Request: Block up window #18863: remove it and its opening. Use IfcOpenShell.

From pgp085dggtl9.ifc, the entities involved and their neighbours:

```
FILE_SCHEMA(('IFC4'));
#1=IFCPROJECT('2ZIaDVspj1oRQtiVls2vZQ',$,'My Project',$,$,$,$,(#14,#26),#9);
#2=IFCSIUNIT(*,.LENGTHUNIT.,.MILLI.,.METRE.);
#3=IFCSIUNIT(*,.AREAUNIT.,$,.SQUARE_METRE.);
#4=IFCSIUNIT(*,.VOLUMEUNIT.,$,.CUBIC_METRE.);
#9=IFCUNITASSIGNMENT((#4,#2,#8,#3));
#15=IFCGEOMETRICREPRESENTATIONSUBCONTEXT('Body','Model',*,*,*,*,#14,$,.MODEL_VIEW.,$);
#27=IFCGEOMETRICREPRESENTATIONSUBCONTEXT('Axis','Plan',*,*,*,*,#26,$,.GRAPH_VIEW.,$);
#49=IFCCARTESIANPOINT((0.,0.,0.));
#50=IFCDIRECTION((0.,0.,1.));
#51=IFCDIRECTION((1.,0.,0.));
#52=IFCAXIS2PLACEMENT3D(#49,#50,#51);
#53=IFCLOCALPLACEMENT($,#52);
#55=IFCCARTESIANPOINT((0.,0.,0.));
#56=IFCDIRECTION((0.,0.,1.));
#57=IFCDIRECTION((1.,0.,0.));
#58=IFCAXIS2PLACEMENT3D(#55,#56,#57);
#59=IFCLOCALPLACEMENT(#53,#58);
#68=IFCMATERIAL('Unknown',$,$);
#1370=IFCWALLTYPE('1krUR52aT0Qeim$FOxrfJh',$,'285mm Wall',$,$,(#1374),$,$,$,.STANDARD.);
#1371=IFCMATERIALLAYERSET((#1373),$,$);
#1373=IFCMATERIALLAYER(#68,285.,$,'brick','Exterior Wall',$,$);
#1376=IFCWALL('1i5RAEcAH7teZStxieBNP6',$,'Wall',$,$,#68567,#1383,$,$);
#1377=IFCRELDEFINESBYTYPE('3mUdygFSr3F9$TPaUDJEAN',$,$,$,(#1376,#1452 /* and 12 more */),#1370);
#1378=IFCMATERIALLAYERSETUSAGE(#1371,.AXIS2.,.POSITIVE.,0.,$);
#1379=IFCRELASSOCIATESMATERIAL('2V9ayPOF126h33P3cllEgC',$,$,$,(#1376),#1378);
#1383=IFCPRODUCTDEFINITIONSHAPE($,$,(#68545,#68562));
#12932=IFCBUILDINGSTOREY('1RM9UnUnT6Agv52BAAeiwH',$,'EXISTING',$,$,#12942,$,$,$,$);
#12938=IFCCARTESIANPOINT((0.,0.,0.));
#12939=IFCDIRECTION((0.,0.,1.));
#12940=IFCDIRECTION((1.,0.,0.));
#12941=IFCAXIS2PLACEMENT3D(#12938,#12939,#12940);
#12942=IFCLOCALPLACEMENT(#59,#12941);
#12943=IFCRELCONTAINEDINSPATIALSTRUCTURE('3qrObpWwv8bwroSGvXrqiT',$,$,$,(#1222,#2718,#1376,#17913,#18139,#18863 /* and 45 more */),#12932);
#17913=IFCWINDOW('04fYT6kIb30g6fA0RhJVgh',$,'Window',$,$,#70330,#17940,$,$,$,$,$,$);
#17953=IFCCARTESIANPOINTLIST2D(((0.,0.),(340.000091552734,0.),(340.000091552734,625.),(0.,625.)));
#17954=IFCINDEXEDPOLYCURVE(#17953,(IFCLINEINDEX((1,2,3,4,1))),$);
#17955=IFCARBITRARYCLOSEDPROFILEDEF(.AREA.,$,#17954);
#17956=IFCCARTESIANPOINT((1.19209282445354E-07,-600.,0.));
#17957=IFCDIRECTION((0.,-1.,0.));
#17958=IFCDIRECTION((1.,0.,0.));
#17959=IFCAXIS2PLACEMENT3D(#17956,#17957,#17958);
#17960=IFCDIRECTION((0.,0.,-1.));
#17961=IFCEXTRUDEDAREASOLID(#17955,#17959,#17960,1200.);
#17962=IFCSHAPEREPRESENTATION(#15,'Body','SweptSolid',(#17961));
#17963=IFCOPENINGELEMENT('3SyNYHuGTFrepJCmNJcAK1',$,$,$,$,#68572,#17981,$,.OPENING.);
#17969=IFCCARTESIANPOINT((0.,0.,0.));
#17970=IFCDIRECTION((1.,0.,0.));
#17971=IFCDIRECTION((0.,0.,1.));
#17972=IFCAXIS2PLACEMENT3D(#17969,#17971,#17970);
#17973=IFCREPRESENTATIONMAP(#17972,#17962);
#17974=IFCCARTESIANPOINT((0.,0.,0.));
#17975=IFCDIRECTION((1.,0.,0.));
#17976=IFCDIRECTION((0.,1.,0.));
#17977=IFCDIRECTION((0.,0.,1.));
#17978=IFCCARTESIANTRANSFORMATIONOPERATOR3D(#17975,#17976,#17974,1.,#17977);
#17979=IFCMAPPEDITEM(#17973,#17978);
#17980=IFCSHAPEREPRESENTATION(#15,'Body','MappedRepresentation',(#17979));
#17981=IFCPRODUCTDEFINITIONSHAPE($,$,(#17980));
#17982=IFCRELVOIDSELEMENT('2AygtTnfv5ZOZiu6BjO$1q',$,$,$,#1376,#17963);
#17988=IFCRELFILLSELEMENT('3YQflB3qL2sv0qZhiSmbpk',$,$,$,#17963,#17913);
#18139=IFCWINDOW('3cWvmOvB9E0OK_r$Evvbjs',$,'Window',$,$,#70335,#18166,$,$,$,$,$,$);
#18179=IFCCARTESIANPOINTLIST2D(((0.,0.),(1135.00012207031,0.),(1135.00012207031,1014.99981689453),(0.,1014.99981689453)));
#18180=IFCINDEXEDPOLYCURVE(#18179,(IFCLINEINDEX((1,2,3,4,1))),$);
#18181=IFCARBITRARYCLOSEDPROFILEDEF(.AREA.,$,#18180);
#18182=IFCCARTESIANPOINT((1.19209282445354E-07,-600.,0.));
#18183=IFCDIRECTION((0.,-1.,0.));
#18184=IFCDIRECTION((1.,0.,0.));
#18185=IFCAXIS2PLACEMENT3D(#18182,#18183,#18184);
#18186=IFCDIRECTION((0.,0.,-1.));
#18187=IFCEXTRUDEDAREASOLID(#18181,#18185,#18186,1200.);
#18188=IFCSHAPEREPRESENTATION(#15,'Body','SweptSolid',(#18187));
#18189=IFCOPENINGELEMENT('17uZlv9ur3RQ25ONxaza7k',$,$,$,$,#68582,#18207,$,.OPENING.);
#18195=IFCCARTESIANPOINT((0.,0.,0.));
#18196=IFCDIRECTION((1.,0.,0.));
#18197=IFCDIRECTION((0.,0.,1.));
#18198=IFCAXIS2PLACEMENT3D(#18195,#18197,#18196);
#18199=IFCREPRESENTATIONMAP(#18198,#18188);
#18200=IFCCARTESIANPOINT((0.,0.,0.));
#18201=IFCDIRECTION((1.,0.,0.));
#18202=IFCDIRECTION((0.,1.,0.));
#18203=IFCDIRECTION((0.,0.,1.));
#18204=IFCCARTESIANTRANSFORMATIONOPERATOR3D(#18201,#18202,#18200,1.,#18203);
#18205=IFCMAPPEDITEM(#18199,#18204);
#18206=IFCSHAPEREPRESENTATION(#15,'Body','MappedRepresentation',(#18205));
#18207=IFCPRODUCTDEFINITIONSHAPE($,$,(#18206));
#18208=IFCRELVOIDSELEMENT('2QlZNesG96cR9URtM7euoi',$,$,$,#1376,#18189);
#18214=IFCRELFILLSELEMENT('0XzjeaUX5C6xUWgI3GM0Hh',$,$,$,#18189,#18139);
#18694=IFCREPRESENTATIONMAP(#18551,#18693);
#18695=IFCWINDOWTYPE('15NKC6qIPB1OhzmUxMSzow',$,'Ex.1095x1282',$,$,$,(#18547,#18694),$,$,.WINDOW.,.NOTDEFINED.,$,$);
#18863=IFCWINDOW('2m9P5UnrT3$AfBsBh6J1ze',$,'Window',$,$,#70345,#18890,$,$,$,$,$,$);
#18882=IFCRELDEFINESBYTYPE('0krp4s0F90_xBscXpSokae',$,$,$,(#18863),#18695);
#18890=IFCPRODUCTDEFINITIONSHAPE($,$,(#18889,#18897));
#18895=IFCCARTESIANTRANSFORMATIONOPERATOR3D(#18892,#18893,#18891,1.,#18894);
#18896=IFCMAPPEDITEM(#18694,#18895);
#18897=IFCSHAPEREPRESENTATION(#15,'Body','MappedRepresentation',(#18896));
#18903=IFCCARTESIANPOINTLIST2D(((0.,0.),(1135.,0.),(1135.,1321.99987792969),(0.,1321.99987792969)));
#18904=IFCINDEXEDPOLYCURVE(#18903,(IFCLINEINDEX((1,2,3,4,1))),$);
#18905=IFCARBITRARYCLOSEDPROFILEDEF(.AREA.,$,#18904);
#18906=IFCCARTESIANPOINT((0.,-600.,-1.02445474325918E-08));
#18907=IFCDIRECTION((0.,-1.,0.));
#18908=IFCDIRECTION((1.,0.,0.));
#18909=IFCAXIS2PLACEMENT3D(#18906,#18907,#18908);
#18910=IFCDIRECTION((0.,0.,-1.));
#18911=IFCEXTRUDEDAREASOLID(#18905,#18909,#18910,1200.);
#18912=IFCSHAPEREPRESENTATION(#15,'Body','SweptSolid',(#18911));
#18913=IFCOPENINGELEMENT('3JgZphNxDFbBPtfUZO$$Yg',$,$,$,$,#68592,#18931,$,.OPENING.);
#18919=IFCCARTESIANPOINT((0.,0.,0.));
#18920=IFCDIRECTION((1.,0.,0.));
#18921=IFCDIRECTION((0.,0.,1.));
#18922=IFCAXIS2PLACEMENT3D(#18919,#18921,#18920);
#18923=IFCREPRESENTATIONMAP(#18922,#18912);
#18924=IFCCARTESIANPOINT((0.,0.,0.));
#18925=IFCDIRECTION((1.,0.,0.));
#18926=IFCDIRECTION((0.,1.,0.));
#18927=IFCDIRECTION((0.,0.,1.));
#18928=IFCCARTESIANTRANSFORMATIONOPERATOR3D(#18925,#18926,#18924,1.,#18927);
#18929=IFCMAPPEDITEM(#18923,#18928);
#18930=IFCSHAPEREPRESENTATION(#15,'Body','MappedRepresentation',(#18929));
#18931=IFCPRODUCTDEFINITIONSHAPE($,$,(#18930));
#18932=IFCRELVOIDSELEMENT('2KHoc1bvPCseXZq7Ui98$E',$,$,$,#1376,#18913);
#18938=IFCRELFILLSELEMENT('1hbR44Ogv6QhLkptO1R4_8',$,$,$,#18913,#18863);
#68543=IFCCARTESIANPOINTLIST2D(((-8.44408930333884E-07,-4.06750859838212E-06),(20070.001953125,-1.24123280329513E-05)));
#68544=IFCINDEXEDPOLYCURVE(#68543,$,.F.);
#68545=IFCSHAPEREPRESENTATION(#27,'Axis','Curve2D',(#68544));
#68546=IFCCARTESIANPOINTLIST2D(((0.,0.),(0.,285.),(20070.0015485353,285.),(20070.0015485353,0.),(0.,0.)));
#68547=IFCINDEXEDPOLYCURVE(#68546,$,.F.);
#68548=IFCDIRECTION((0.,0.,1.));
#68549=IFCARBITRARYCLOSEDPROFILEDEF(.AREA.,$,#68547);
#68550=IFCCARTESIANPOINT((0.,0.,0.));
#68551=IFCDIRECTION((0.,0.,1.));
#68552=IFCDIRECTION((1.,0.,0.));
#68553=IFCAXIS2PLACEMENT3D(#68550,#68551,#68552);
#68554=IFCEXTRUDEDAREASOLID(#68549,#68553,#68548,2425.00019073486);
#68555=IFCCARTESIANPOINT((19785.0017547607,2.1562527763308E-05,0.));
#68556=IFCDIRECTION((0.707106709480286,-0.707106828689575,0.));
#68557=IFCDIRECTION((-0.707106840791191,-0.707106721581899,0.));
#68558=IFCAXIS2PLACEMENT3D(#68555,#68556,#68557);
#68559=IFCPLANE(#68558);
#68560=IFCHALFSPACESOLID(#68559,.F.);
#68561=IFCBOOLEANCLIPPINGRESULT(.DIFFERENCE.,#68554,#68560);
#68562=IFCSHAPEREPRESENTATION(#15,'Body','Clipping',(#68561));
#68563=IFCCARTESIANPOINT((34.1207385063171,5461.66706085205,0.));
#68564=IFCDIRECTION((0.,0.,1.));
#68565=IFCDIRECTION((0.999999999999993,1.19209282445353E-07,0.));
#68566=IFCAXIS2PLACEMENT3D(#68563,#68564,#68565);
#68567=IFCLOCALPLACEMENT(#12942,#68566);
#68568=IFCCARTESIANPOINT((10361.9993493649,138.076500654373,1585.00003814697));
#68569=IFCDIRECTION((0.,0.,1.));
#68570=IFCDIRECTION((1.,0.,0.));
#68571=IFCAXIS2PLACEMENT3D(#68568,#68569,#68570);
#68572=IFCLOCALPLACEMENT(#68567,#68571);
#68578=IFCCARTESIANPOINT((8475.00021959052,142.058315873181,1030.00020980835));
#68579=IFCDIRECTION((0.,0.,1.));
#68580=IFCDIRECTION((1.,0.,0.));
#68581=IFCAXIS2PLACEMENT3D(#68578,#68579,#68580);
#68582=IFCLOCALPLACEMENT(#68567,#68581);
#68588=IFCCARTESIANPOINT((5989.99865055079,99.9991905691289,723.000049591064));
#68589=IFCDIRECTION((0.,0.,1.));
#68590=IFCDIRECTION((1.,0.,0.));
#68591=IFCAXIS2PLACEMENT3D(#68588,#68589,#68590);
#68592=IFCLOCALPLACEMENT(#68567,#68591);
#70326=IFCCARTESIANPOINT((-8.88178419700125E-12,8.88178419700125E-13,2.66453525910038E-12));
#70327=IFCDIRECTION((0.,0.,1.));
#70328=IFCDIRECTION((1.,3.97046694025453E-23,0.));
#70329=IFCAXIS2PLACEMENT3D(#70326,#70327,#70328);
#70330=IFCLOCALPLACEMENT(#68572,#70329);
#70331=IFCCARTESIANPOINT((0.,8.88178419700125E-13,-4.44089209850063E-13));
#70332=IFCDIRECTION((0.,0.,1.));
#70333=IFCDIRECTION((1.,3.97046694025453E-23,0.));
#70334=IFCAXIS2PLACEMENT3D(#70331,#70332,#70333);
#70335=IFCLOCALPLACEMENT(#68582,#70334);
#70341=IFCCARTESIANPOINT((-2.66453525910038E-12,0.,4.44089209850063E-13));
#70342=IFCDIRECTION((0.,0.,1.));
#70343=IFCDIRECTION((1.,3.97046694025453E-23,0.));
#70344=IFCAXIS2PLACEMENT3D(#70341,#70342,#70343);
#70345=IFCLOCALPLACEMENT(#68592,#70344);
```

```python
import ifcopenshell
import ifcopenshell.api.feature
import ifcopenshell.api.root
import ifcopenshell.geom
import ifcopenshell.util.shape

model = ifcopenshell.open("pgp085dggtl9.ifc")
settings = ifcopenshell.geom.settings()


def volume(element):
    """Net volume in cubic metres, openings subtracted."""
    shape = ifcopenshell.geom.create_shape(settings, element)
    return ifcopenshell.util.shape.get_volume(shape.geometry)


window = model.by_guid("2m9P5UnrT3$AfBsBh6J1ze")
opening = window.FillsVoids[0].RelatingOpeningElement
wall = opening.VoidsElements[0].RelatingBuildingElement
before = volume(wall)

ifcopenshell.api.root.remove_product(model, product=window)
ifcopenshell.api.feature.remove_feature(model, feature=opening)

after = volume(wall)

print(f"wall volume {before:.3f} -> {after:.3f} m3")

model.write("pgp085dggtl9_updated.ifc")
```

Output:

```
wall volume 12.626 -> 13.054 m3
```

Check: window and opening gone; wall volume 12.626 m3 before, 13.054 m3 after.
